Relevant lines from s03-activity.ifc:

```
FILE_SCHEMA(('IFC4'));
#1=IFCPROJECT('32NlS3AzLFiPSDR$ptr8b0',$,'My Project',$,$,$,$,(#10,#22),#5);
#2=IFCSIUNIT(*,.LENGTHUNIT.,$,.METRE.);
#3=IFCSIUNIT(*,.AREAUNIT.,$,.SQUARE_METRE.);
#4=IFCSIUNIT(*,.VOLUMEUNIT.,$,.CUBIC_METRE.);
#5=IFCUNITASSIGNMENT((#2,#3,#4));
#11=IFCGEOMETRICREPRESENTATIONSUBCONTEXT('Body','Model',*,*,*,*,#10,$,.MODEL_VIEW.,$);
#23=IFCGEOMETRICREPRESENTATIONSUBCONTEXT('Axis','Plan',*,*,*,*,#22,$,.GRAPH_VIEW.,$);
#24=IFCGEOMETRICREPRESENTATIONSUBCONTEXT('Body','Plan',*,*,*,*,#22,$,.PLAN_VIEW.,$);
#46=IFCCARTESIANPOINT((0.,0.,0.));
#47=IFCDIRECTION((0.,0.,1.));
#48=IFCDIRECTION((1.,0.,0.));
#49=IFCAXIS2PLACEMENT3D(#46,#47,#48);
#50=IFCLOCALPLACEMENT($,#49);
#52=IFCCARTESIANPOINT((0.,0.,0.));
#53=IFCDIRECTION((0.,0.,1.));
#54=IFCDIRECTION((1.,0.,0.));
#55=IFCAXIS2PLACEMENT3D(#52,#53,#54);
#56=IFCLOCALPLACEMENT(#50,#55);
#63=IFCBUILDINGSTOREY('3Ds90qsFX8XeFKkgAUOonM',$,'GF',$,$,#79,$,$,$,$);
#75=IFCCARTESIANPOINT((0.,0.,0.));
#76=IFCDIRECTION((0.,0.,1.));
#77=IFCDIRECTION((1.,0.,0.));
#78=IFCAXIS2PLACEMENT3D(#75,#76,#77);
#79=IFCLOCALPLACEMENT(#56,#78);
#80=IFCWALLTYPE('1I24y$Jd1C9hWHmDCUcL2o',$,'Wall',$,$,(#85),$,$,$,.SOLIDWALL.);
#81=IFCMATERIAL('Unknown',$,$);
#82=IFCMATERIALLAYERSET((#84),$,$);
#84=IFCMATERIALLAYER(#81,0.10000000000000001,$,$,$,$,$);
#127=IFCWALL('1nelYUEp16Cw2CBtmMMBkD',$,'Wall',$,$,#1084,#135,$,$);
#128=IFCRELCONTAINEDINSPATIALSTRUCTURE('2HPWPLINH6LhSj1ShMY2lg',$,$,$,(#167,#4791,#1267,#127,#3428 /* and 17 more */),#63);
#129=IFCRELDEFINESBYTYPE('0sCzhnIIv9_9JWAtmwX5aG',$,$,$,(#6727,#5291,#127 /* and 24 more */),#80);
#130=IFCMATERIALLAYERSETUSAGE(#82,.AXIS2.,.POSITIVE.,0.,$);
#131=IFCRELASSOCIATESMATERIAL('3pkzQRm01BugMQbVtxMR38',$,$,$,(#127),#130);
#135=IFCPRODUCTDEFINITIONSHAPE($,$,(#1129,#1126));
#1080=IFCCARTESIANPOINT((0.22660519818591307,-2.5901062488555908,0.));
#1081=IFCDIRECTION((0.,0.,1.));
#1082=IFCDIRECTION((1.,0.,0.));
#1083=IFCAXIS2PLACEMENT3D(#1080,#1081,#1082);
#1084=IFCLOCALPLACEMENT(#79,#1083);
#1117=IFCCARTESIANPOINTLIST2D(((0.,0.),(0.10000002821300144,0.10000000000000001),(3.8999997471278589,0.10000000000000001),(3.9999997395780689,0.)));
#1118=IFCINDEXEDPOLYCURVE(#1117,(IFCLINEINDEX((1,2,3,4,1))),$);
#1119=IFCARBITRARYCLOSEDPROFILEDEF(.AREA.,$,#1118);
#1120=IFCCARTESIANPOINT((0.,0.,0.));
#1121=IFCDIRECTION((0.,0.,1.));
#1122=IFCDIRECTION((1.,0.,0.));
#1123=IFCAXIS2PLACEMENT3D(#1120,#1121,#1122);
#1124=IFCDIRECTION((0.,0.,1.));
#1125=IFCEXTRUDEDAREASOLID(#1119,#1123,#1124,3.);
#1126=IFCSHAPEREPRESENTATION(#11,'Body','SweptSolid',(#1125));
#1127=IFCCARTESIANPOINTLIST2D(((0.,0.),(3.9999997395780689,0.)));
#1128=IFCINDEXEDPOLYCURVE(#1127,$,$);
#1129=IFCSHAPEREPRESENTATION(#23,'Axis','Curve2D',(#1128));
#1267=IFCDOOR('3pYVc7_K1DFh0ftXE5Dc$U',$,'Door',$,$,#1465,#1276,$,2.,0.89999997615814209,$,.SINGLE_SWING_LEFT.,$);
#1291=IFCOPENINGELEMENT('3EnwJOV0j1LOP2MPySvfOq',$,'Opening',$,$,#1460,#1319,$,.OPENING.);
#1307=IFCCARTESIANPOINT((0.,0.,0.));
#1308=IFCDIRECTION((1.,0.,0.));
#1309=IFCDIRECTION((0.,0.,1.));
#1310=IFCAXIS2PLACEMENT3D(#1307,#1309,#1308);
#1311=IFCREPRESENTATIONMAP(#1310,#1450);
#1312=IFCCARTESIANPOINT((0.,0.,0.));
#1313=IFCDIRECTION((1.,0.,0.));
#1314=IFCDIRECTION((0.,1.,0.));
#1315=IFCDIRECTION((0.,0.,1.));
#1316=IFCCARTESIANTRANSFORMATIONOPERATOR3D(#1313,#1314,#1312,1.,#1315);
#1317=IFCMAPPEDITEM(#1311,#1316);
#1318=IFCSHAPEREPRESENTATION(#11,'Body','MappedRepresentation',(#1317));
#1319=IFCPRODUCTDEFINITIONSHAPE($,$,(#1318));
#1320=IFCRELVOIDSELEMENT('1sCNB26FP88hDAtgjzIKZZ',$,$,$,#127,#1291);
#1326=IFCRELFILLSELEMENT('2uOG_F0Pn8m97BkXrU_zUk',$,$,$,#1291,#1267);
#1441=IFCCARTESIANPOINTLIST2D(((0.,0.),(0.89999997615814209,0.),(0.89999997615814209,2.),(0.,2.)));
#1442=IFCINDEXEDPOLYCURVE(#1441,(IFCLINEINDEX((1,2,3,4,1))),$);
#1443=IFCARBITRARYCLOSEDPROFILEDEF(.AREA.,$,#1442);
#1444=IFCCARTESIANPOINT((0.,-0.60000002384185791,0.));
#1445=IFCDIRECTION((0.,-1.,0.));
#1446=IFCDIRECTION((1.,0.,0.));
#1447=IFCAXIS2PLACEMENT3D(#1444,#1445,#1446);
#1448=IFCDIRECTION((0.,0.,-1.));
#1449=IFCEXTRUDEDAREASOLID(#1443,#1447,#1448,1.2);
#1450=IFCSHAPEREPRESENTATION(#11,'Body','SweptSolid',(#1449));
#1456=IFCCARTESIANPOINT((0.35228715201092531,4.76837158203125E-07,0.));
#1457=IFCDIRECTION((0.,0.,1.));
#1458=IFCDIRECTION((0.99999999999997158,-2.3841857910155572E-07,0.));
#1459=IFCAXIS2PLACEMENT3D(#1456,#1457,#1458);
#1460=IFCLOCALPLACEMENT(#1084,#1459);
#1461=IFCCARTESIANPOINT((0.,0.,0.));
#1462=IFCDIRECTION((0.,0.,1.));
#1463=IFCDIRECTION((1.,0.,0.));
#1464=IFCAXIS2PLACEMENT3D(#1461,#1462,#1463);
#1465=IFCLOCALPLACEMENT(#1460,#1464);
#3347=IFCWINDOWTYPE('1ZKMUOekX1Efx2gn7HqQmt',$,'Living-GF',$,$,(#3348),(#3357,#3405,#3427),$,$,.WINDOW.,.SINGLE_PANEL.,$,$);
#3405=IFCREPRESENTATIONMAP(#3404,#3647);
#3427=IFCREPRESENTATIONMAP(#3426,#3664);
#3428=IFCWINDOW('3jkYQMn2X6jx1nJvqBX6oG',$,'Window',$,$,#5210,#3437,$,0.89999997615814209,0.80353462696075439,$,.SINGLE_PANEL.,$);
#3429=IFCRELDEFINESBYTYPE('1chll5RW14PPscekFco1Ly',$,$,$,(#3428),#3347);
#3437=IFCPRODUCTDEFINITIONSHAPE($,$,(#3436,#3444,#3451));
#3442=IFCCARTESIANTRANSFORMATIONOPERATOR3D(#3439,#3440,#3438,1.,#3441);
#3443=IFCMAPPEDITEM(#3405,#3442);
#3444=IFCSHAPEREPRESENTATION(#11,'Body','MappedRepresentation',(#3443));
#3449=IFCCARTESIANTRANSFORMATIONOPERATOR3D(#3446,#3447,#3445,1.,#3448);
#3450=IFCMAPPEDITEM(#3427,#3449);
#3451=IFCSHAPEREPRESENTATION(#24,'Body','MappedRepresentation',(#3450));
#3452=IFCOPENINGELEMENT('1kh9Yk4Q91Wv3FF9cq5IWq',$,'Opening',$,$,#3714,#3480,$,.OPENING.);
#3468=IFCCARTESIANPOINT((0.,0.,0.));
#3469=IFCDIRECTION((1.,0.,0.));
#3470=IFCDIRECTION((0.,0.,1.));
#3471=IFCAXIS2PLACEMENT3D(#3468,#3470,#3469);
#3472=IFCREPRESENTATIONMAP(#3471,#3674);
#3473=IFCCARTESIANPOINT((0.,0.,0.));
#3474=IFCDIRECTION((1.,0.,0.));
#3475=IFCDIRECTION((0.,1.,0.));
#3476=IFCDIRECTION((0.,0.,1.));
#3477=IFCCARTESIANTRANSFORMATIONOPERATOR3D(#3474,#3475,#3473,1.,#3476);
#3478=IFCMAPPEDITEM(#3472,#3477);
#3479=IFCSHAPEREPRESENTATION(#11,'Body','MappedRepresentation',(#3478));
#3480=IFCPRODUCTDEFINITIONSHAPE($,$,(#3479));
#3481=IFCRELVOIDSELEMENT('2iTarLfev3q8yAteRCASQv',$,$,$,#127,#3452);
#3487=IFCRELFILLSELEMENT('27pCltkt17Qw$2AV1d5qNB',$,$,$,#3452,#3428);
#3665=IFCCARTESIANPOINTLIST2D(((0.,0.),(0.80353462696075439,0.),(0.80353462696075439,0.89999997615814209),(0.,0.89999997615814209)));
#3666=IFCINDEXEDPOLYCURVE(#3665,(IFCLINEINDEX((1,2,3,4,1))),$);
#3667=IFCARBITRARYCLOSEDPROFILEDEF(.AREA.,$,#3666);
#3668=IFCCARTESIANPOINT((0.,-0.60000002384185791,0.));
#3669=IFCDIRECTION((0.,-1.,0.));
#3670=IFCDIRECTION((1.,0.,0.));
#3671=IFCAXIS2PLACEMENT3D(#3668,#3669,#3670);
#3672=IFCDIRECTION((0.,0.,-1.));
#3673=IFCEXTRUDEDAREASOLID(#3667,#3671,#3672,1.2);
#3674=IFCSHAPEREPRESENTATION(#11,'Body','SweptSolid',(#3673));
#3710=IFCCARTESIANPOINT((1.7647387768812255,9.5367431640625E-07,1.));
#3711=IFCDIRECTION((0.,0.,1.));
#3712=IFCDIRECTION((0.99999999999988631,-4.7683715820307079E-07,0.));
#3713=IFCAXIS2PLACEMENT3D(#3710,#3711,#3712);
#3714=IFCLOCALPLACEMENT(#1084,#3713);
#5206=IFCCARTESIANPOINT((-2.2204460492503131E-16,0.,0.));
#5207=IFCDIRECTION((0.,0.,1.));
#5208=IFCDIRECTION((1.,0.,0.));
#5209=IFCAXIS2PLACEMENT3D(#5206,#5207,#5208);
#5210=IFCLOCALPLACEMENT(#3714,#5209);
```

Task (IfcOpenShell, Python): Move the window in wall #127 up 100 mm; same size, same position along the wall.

```python
import numpy as np
import ifcopenshell
import ifcopenshell.api.geometry
import ifcopenshell.util.placement
import ifcopenshell.util.unit

model = ifcopenshell.open("s03-activity.ifc")
unit_scale = ifcopenshell.util.unit.calculate_unit_scale(model)

window = model.by_guid("3jkYQMn2X6jx1nJvqBX6oG")
opening = window.FillsVoids[0].RelatingOpeningElement
dz = 0.1 / unit_scale

shift = np.array([0.0, 0.0, dz])
# The window is placed relative to its opening, so it follows when the opening moves.
matrix = ifcopenshell.util.placement.get_local_placement(opening.ObjectPlacement)
matrix[:3, 3] += shift
ifcopenshell.api.geometry.edit_object_placement(
    model, product=opening, matrix=matrix, is_si=False, should_transform_children=True
)

print(f"moved by {dz * unit_scale:+.3f} m")

model.write("s03-activity_updated.ifc")
```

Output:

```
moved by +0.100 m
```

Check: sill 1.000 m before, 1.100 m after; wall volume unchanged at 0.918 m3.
